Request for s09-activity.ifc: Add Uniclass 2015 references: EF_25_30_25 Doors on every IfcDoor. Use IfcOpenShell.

First a look at what the model holds.

```python
import ifcopenshell

model = ifcopenshell.open("s09-activity.ifc")
print(model.schema)
print("classifications:", [c.Name for c in model.by_type("IfcClassification")])
for ifc_class in ("IfcDoor", "IfcRoof", "IfcStair", "IfcWall", "IfcWindow"):
    print(ifc_class, len(model.by_type(ifc_class)))
```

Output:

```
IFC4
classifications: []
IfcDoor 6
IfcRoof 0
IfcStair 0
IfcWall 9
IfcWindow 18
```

```python
import ifcopenshell
import ifcopenshell.api.classification

model = ifcopenshell.open("s09-activity.ifc")

system = ifcopenshell.api.classification.add_classification(model, classification="Uniclass 2015")

codes = {
    "IfcDoor": ("EF_25_30_25", "Doors"),
}
for ifc_class, (code, name) in codes.items():
    products = model.by_type(ifc_class)
    ifcopenshell.api.classification.add_reference(
        model, products=products, classification=system, identification=code, name=name
    )
    print(code, len(products))

model.write("s09-activity_rev.ifc")
```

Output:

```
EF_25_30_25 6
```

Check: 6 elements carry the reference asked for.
